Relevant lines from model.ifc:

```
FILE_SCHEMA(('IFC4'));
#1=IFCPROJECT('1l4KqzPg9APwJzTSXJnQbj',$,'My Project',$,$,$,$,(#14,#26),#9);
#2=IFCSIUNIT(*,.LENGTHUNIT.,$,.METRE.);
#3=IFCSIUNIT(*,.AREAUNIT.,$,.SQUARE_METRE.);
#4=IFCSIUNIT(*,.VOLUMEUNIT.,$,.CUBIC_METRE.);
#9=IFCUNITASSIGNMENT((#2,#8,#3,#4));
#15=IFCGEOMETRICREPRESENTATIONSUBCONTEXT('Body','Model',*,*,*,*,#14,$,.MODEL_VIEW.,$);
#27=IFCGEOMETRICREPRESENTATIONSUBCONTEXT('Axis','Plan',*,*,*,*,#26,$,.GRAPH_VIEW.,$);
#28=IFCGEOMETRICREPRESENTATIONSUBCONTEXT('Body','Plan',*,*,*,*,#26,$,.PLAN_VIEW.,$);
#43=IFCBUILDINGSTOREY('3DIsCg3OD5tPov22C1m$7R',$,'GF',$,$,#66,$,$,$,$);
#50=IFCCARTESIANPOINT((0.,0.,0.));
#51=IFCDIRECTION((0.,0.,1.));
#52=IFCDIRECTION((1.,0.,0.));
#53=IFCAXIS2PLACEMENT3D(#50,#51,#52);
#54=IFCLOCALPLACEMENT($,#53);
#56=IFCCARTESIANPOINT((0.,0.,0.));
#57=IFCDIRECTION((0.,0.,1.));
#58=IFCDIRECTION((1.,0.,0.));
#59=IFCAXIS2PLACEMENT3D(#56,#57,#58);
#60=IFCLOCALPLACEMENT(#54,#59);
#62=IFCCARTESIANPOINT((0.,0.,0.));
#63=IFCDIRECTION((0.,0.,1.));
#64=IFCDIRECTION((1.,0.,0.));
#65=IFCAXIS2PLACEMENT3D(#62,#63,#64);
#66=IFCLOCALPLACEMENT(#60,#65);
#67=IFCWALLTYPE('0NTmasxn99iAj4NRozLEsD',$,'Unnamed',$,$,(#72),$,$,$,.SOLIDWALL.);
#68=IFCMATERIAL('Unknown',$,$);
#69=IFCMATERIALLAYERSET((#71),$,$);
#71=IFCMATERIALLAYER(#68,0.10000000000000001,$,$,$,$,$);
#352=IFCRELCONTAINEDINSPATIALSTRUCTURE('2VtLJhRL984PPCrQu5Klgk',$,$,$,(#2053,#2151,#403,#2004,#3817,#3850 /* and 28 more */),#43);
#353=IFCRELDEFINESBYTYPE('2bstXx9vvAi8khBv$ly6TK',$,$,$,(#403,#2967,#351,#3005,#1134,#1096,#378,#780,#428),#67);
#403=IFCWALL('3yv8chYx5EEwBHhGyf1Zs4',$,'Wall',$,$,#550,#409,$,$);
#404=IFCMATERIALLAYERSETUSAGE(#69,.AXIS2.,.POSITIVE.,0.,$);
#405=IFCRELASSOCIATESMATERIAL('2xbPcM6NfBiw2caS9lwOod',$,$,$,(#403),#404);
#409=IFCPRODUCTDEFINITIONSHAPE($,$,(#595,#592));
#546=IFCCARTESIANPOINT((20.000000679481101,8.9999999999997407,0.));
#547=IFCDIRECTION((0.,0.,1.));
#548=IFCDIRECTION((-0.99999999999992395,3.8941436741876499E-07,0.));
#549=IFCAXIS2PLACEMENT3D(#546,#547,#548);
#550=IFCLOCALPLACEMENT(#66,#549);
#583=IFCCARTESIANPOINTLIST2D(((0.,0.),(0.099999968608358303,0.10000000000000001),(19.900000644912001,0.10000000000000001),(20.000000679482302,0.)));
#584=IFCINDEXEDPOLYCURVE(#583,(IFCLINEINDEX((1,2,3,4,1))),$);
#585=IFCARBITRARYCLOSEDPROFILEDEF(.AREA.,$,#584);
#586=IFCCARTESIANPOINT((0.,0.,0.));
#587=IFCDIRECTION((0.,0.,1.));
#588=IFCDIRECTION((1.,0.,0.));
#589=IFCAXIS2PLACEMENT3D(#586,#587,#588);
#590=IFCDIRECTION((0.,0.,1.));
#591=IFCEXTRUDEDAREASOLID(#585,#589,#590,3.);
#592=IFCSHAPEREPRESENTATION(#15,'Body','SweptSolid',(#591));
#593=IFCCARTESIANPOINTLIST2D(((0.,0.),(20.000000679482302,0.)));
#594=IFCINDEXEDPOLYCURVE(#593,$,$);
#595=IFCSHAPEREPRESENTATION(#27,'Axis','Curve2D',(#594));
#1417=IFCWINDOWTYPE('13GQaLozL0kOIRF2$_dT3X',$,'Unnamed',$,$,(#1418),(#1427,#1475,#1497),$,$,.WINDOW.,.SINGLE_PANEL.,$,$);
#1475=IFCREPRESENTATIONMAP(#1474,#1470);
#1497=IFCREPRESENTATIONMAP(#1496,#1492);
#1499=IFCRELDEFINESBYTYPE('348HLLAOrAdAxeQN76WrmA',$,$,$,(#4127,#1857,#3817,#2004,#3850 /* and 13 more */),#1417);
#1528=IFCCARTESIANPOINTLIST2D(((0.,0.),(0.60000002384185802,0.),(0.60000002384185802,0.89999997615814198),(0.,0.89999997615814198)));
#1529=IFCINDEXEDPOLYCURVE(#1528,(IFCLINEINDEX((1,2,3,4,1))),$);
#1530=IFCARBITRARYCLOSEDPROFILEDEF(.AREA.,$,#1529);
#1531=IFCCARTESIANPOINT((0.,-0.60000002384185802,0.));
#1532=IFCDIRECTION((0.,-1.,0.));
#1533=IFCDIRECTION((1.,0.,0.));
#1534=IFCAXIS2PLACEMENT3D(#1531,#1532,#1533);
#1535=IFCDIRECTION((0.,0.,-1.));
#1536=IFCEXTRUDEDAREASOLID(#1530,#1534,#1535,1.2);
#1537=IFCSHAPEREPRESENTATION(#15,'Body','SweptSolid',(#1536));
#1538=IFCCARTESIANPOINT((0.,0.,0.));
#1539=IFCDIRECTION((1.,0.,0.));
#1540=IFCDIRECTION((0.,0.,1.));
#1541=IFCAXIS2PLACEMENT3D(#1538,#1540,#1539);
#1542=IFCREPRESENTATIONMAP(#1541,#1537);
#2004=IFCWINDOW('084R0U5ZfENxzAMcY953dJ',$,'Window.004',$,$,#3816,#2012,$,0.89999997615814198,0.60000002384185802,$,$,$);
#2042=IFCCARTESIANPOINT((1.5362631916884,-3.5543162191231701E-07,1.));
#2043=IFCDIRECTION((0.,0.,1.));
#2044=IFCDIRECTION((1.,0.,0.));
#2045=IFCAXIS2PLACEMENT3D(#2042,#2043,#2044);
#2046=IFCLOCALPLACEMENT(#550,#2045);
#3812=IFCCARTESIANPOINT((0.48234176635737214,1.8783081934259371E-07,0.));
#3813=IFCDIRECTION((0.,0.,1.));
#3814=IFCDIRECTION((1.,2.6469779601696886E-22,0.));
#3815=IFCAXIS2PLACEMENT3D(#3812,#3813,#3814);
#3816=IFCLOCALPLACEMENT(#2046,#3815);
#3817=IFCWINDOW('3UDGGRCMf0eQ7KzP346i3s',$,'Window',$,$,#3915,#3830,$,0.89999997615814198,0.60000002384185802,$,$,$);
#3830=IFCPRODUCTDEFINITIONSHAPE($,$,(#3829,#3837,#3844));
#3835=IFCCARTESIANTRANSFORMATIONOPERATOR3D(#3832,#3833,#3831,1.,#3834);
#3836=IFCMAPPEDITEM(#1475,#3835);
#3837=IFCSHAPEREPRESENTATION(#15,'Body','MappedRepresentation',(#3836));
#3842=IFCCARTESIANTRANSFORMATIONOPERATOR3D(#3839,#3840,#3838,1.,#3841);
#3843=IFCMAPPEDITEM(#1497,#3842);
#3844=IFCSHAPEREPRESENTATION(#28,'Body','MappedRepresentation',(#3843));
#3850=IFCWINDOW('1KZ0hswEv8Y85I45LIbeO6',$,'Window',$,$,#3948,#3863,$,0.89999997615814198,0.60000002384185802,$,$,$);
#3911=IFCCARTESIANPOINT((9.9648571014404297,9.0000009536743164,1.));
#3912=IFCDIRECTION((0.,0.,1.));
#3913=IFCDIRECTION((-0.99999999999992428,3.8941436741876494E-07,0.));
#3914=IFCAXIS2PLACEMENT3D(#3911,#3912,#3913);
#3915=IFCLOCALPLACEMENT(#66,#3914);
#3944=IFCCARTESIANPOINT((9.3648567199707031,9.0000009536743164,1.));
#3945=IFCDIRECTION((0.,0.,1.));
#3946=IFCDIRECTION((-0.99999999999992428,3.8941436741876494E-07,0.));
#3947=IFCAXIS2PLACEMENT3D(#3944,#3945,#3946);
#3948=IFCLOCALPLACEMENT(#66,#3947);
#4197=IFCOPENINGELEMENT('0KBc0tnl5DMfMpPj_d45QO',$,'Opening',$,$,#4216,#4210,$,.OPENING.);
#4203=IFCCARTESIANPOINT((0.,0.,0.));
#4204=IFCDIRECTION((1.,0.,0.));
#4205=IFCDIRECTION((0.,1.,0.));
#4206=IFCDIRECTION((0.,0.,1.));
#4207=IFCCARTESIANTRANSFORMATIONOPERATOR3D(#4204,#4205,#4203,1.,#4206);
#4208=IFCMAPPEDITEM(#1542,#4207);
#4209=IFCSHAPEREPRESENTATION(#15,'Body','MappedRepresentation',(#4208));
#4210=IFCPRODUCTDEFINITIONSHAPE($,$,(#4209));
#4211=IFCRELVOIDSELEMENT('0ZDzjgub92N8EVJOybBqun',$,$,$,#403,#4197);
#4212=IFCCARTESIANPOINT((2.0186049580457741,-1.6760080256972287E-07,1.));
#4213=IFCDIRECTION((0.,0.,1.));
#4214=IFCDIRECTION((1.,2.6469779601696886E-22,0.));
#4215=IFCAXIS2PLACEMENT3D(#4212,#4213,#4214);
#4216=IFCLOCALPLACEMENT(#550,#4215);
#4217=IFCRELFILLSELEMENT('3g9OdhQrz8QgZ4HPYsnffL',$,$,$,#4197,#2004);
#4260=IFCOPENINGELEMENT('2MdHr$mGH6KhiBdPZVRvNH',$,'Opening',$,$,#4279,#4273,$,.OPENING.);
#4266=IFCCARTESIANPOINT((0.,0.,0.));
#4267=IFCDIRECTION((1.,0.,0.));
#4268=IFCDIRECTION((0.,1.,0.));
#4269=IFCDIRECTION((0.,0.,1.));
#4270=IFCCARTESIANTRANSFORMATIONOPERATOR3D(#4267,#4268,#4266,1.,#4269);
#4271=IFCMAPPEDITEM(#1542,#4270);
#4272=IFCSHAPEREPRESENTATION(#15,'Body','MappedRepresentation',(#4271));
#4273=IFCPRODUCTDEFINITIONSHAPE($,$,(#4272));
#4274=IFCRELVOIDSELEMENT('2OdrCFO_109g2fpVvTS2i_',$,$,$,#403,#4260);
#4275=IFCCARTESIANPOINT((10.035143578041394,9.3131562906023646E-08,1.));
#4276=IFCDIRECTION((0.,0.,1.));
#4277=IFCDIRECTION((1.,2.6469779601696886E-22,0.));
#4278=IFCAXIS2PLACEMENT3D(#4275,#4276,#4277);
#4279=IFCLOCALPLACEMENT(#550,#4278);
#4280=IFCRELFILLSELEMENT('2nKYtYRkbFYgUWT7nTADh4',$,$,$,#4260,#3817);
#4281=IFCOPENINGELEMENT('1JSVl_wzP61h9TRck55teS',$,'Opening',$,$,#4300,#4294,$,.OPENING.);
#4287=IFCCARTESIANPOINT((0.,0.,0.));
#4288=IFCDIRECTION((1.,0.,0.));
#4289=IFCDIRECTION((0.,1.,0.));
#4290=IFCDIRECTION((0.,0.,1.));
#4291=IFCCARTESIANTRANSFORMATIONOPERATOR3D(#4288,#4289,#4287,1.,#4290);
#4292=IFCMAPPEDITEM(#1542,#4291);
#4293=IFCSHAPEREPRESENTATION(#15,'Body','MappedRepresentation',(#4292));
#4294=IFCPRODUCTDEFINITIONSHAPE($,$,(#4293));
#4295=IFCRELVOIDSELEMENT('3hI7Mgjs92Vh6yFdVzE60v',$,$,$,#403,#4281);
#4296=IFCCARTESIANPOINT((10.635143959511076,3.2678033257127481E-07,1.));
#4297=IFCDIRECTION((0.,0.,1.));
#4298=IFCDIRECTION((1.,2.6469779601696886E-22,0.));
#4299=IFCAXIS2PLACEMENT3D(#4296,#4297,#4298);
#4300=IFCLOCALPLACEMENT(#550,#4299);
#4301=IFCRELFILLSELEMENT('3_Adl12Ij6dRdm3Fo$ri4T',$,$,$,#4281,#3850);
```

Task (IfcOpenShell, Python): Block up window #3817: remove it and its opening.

```python
import ifcopenshell
import ifcopenshell.api.feature
import ifcopenshell.api.root
import ifcopenshell.geom
import ifcopenshell.util.shape

model = ifcopenshell.open("model.ifc")
settings = ifcopenshell.geom.settings()


def volume(element):
    """Net volume in cubic metres, openings subtracted."""
    shape = ifcopenshell.geom.create_shape(settings, element)
    return ifcopenshell.util.shape.get_volume(shape.geometry)


window = model.by_guid("3UDGGRCMf0eQ7KzP346i3s")
opening = window.FillsVoids[0].RelatingOpeningElement
wall = opening.VoidsElements[0].RelatingBuildingElement
before = volume(wall)

ifcopenshell.api.root.remove_product(model, product=window)
ifcopenshell.api.feature.remove_feature(model, feature=opening)

after = volume(wall)

print(f"wall volume {before:.3f} -> {after:.3f} m3")

model.write("model_updated.ifc")
```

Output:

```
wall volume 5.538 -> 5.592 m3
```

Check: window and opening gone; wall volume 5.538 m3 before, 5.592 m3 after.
